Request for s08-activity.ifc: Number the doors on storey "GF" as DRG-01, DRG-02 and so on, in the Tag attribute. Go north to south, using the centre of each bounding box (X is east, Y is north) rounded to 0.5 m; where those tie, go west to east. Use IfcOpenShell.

First a look at what the model holds.

```python
import ifcopenshell
import ifcopenshell.util.element
import ifcopenshell.util.placement

model = ifcopenshell.open("s08-activity.ifc")
print(model.schema)
storey = next(s for s in model.by_type("IfcBuildingStorey") if s.Name == "GF")
doors = [e for e in ifcopenshell.util.element.get_decomposition(storey) if e.is_a("IfcDoor")]
for e in sorted(doors, key=lambda e: e.id()):
    origin = ifcopenshell.util.placement.get_local_placement(e.ObjectPlacement)[:3, 3]
    print(e.id(), e.Tag, e.Name, origin.round(2) + 0.0, sep=" | ")
```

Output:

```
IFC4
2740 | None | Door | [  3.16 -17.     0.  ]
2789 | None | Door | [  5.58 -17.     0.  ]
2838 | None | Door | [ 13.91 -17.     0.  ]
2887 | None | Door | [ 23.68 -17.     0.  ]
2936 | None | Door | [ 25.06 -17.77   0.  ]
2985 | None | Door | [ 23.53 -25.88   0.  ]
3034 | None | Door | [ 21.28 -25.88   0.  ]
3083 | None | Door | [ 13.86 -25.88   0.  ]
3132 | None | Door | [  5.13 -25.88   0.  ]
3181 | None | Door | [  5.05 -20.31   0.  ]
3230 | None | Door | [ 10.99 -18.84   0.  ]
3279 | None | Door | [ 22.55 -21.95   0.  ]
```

```python
import ifcopenshell
import ifcopenshell.geom
import ifcopenshell.util.element
import ifcopenshell.util.shape

model = ifcopenshell.open("s08-activity.ifc")
settings = ifcopenshell.geom.settings()
settings.set("use-world-coords", True)


def centre(element):
    shape = ifcopenshell.geom.create_shape(settings, element)
    return ifcopenshell.util.shape.get_bbox_centroid(shape.geometry)


storey = next(s for s in model.by_type("IfcBuildingStorey") if s.Name == "GF")
doors = [e for e in ifcopenshell.util.element.get_decomposition(storey) if e.is_a("IfcDoor")]

# Insertion points can sit at a corner or the storey origin, so sort by the geometry (in metres).
centres = {e: centre(e) for e in doors}
doors.sort(key=lambda e: (-round(centres[e][1] / 0.5), centres[e][0]))

for i, e in enumerate(doors, start=1):
    number = f"DRG-{i:02d}"
    e.Tag = number
    print(e.id(), number)

model.write("s08-activity_edited.ifc")
```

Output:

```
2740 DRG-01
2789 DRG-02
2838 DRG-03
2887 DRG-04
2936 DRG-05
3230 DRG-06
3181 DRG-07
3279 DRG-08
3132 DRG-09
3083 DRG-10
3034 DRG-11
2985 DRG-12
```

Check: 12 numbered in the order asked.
